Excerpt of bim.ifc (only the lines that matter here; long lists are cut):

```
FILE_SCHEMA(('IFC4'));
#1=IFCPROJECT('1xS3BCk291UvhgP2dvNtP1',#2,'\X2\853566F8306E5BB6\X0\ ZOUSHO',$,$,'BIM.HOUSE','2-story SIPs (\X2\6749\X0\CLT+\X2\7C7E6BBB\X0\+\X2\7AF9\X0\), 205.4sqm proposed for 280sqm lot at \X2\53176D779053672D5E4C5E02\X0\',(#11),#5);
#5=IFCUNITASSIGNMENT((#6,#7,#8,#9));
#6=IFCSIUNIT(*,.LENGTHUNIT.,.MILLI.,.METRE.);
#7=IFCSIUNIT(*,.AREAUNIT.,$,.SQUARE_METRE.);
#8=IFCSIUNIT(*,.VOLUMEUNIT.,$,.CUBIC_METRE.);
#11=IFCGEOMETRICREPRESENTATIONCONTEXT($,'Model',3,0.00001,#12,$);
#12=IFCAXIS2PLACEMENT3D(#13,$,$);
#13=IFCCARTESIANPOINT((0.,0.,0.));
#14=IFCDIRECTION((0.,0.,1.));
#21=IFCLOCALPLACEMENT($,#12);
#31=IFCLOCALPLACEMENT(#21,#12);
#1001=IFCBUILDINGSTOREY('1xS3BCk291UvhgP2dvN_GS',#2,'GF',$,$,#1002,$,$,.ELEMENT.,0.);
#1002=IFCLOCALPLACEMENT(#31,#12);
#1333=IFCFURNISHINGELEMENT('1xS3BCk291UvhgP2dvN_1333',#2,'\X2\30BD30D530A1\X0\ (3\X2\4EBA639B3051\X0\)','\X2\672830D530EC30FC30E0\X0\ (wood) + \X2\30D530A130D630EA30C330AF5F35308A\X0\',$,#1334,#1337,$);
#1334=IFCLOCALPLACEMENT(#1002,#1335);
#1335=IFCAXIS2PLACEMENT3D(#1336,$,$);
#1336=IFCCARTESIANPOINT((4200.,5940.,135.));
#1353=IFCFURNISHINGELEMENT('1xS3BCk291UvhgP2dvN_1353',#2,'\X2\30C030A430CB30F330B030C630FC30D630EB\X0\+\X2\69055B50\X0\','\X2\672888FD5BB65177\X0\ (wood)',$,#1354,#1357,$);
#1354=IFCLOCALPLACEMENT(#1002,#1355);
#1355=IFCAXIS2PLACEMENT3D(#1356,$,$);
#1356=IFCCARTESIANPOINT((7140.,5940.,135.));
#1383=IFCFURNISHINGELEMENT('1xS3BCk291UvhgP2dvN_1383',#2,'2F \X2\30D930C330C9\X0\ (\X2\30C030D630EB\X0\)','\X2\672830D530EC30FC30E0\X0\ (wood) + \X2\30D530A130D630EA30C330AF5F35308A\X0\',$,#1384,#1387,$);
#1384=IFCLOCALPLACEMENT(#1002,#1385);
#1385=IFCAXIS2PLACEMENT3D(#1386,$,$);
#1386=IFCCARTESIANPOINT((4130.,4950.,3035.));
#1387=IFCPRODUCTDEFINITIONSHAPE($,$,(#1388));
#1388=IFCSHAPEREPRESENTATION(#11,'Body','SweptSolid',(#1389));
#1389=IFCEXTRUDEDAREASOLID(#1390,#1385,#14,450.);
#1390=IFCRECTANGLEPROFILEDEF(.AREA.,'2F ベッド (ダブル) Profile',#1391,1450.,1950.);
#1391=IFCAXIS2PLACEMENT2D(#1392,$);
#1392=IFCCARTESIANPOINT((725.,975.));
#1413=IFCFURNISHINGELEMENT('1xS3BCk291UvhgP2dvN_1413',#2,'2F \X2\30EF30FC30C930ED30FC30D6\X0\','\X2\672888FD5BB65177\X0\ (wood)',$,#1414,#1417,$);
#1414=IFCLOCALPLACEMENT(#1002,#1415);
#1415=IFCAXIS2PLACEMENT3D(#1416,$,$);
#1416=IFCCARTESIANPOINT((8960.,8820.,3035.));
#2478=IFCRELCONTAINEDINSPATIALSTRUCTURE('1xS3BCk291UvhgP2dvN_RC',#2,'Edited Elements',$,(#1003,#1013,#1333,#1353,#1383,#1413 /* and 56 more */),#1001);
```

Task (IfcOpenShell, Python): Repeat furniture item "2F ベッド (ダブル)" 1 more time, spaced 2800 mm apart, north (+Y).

```python
import numpy as np
import ifcopenshell
import ifcopenshell.api.geometry
import ifcopenshell.api.root
import ifcopenshell.util.element
import ifcopenshell.util.placement
import ifcopenshell.util.unit

model = ifcopenshell.open("bim.ifc")
unit_scale = ifcopenshell.util.unit.calculate_unit_scale(model)


def reuse_history(source, copy):
    """copy_class also copies each property set's owner history, people and application; keep the originals."""
    for rel in copy.IsDefinedBy:
        if rel.is_a("IfcRelDefinesByProperties") and (history := rel.RelatingPropertyDefinition.OwnerHistory):
            rel.RelatingPropertyDefinition.OwnerHistory = source.OwnerHistory
            ifcopenshell.util.element.remove_deep2(model, history)


source = model.by_guid("1xS3BCk291UvhgP2dvN_1383")
base = ifcopenshell.util.placement.get_local_placement(source.ObjectPlacement)
step = np.array([0.0, 1.0, 0.0]) * 2.8 / unit_scale

for i in range(1, 2):
    copy = ifcopenshell.api.root.copy_class(model, product=source)
    copy.Representation = ifcopenshell.util.element.copy_deep(
        model, source.Representation, exclude=["IfcGeometricRepresentationContext", "IfcRepresentationMap"]
    )
    reuse_history(source, copy)
    matrix = base.copy()
    matrix[:3, 3] += i * step
    print("added at", matrix[:3, 3].round(3) + 0.0)
    ifcopenshell.api.geometry.edit_object_placement(model, product=copy, matrix=matrix, is_si=False)

model.write("bim_rev.ifc")
```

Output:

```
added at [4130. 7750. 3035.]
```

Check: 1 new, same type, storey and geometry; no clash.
